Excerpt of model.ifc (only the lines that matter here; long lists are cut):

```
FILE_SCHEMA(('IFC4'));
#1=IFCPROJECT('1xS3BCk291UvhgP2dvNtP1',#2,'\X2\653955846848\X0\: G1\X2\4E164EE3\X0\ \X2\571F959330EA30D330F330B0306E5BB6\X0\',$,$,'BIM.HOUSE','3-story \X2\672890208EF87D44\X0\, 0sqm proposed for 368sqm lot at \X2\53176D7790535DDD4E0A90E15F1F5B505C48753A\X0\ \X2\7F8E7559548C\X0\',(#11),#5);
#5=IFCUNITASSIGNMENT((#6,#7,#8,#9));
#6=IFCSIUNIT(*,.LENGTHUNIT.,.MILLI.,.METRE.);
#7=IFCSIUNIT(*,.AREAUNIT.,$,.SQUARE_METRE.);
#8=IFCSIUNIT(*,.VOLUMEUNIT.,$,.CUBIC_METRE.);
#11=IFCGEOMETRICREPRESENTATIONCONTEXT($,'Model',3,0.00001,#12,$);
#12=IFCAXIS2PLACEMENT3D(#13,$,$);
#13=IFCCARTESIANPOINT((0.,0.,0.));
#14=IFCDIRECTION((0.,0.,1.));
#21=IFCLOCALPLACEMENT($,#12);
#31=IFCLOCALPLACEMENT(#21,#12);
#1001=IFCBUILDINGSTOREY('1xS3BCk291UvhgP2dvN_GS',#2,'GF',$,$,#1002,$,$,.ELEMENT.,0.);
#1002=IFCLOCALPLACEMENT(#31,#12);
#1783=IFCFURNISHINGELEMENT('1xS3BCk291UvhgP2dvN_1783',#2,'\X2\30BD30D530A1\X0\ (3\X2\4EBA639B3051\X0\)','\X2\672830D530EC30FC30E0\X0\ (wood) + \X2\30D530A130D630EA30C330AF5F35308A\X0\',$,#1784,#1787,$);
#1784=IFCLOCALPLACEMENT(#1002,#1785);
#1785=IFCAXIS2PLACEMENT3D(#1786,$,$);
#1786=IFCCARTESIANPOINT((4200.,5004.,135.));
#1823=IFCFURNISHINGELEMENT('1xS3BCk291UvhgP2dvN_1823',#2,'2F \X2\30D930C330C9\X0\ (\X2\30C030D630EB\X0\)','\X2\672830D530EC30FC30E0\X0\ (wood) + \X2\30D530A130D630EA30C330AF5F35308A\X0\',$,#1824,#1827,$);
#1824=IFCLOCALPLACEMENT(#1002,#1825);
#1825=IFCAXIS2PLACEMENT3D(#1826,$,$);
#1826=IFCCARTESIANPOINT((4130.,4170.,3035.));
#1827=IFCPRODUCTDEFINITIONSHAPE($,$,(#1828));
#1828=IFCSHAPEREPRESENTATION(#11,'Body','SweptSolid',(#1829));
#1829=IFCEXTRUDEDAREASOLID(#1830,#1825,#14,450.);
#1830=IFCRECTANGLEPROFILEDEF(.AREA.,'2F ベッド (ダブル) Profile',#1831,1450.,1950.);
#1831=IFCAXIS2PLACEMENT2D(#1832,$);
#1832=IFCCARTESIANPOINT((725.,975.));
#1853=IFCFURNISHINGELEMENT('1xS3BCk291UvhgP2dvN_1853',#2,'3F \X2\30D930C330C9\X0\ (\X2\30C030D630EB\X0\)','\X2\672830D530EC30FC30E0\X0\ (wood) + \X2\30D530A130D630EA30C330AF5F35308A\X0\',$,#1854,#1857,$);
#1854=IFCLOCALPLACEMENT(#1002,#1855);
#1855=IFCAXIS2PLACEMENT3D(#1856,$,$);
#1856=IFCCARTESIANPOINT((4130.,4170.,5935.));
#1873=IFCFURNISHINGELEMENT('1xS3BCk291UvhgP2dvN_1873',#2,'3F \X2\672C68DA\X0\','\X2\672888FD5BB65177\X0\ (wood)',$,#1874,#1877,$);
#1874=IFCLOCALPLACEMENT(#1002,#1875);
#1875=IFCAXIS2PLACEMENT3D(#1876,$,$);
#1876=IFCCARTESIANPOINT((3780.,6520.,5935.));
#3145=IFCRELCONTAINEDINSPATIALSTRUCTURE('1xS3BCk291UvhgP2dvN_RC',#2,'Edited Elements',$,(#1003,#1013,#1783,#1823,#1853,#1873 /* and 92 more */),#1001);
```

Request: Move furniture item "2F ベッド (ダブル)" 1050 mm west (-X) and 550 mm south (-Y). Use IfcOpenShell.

```python
import ifcopenshell
import ifcopenshell.api.geometry
import ifcopenshell.util.placement
import ifcopenshell.util.unit

model = ifcopenshell.open("model.ifc")
unit_scale = ifcopenshell.util.unit.calculate_unit_scale(model)

item = model.by_guid("1xS3BCk291UvhgP2dvN_1823")
matrix = ifcopenshell.util.placement.get_local_placement(item.ObjectPlacement)
matrix[0, 3] -= 1.05 / unit_scale
matrix[1, 3] -= 0.55 / unit_scale
ifcopenshell.api.geometry.edit_object_placement(model, product=item, matrix=matrix, is_si=False)

print(ifcopenshell.util.placement.get_local_placement(item.ObjectPlacement).round(3) + 0.0)

model.write("model_updated.ifc")
```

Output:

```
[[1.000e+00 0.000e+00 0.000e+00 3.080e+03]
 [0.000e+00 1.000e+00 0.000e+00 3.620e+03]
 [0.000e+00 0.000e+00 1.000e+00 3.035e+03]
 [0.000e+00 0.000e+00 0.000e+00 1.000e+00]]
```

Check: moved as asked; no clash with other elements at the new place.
